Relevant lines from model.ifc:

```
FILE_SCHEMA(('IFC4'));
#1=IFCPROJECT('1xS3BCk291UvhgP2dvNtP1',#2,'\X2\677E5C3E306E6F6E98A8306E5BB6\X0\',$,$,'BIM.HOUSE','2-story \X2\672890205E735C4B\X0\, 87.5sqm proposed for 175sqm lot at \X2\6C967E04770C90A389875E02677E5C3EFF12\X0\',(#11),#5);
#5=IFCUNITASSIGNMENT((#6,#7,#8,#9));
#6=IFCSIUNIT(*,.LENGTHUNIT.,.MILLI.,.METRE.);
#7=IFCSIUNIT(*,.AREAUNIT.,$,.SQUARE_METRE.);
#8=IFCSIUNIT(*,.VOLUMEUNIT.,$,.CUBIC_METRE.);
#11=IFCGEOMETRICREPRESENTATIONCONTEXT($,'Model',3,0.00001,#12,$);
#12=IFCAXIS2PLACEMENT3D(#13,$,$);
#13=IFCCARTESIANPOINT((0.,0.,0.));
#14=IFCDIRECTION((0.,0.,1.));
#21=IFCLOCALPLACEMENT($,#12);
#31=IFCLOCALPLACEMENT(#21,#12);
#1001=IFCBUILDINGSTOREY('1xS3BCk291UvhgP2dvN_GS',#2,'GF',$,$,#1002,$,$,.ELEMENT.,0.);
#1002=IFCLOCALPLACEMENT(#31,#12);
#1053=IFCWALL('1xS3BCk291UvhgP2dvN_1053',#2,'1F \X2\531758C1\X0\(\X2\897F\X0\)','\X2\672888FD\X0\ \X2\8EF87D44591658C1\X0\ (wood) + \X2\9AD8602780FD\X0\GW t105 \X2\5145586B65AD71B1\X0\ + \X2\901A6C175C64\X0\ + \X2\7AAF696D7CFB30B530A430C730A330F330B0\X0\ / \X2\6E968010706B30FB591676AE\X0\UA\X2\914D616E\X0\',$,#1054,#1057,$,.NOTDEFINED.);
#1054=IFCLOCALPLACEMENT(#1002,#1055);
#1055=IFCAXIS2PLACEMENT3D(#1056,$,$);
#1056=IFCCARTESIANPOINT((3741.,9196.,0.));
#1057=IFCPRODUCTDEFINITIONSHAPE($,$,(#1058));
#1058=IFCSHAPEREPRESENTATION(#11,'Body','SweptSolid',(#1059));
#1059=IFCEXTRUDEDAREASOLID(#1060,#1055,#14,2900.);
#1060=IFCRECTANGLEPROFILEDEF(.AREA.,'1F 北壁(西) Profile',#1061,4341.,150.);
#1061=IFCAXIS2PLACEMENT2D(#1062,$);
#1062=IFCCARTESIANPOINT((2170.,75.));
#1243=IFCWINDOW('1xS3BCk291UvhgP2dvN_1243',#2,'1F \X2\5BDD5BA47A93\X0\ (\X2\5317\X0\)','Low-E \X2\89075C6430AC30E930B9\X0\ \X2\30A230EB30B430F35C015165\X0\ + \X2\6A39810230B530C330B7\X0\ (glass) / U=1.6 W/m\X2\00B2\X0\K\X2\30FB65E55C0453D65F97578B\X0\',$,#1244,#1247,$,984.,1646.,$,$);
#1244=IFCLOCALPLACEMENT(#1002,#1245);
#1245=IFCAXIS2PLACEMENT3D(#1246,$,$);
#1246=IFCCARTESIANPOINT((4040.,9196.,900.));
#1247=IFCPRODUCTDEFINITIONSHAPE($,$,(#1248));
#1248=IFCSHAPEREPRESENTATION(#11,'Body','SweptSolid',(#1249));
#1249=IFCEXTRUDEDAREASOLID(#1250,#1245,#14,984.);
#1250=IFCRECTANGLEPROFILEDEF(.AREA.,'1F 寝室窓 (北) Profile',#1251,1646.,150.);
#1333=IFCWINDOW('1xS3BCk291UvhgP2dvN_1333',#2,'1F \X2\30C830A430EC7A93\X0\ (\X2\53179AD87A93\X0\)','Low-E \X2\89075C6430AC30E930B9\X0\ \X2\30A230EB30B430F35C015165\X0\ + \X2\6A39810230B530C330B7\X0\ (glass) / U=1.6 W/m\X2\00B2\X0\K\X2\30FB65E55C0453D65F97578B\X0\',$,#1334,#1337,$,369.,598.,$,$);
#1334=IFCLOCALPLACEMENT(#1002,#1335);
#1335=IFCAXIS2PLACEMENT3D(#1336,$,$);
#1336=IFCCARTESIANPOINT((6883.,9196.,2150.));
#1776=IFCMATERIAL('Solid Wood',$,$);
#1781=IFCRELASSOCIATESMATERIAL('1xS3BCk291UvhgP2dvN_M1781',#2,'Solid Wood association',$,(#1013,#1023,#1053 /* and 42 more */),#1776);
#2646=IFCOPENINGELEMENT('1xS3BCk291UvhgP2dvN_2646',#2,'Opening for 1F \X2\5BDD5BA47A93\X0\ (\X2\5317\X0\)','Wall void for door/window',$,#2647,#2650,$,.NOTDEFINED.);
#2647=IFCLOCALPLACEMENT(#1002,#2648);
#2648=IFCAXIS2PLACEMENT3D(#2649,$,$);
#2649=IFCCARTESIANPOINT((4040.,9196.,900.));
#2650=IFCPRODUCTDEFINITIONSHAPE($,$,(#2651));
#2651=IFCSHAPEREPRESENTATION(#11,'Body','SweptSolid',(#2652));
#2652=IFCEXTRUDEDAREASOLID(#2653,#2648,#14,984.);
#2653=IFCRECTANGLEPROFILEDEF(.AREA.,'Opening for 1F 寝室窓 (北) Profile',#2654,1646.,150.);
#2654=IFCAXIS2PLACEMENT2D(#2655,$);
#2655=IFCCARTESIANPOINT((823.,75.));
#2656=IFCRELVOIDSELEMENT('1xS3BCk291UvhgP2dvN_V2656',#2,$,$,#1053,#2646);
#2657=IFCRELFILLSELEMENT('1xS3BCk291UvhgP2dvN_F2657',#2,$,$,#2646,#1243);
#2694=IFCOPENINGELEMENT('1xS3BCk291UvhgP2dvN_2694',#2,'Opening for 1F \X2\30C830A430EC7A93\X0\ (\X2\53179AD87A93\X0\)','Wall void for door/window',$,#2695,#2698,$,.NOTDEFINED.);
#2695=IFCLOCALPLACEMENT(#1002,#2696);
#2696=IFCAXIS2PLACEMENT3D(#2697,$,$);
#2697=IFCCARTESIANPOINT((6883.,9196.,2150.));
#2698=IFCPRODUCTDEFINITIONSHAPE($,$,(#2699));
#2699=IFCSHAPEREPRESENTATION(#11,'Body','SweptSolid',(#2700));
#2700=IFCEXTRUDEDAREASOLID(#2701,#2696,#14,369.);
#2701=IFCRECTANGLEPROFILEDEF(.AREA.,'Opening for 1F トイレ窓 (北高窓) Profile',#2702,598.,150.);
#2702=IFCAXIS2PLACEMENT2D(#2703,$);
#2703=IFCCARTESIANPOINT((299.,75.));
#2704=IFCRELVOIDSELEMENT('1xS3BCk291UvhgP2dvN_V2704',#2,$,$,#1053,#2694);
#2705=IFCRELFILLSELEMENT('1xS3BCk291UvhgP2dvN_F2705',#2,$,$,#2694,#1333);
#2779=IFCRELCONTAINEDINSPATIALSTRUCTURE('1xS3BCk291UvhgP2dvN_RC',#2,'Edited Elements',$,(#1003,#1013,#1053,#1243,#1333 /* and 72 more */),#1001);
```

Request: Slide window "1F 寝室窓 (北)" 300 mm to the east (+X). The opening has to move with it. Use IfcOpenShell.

```python
import ifcopenshell
import ifcopenshell.api.geometry
import ifcopenshell.util.placement

model = ifcopenshell.open("model.ifc")

window = model.by_guid("1xS3BCk291UvhgP2dvN_1243")
opening = window.FillsVoids[0].RelatingOpeningElement
wall = opening.VoidsElements[0].RelatingBuildingElement

wall_matrix = ifcopenshell.util.placement.get_local_placement(wall.ObjectPlacement)
shift = wall_matrix[:3, 0] * 300.0
before = ifcopenshell.util.placement.get_local_placement(window.ObjectPlacement)[:3, 3].copy()

# The window is not placed relative to its opening, so move both.
for product in (opening, window):
    matrix = ifcopenshell.util.placement.get_local_placement(product.ObjectPlacement)
    matrix[:3, 3] += shift
    ifcopenshell.api.geometry.edit_object_placement(model, product=product, matrix=matrix, is_si=False)

after = ifcopenshell.util.placement.get_local_placement(window.ObjectPlacement)[:3, 3]
print("window moved by", (after - before).round(3) + 0.0)

model.write("model_rev.ifc")
```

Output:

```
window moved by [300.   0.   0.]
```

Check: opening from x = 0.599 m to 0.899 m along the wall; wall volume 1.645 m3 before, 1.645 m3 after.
